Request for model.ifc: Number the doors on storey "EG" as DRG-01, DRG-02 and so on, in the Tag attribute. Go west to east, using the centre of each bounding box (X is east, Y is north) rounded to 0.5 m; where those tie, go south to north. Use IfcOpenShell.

First a look at what the model holds.

```python
import ifcopenshell
import ifcopenshell.util.element
import ifcopenshell.util.placement

model = ifcopenshell.open("model.ifc")
print(model.schema)
storey = next(s for s in model.by_type("IfcBuildingStorey") if s.Name == "EG")
doors = [e for e in ifcopenshell.util.element.get_decomposition(storey) if e.is_a("IfcDoor")]
for e in sorted(doors, key=lambda e: e.id()):
    origin = ifcopenshell.util.placement.get_local_placement(e.ObjectPlacement)[:3, 3]
    print(e.id(), e.Tag, e.Name, origin.round(2) + 0.0, sep=" | ")
```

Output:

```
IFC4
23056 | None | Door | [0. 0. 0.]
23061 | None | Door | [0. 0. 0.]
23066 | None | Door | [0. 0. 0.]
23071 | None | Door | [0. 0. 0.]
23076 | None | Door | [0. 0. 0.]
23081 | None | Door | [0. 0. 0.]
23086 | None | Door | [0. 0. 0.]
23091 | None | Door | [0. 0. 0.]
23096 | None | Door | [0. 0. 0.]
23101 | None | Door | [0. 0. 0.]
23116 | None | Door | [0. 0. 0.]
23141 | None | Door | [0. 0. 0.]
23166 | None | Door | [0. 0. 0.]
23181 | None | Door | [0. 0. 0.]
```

```python
import ifcopenshell
import ifcopenshell.geom
import ifcopenshell.util.element
import ifcopenshell.util.shape

model = ifcopenshell.open("model.ifc")
settings = ifcopenshell.geom.settings()
settings.set("use-world-coords", True)


def centre(element):
    shape = ifcopenshell.geom.create_shape(settings, element)
    return ifcopenshell.util.shape.get_bbox_centroid(shape.geometry)


storey = next(s for s in model.by_type("IfcBuildingStorey") if s.Name == "EG")
doors = [e for e in ifcopenshell.util.element.get_decomposition(storey) if e.is_a("IfcDoor")]

# Insertion points can sit at a corner or the storey origin, so sort by the geometry (in metres).
centres = {e: centre(e) for e in doors}
doors.sort(key=lambda e: (round(centres[e][0] / 0.5), centres[e][1]))

for i, e in enumerate(doors, start=1):
    number = f"DRG-{i:02d}"
    e.Tag = number
    print(e.id(), number)

model.write("model_edited.ifc")
```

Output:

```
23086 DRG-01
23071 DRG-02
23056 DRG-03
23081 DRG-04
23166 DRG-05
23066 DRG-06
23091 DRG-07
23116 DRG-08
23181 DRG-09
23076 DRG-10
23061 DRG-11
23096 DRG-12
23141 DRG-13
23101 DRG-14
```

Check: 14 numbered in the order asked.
